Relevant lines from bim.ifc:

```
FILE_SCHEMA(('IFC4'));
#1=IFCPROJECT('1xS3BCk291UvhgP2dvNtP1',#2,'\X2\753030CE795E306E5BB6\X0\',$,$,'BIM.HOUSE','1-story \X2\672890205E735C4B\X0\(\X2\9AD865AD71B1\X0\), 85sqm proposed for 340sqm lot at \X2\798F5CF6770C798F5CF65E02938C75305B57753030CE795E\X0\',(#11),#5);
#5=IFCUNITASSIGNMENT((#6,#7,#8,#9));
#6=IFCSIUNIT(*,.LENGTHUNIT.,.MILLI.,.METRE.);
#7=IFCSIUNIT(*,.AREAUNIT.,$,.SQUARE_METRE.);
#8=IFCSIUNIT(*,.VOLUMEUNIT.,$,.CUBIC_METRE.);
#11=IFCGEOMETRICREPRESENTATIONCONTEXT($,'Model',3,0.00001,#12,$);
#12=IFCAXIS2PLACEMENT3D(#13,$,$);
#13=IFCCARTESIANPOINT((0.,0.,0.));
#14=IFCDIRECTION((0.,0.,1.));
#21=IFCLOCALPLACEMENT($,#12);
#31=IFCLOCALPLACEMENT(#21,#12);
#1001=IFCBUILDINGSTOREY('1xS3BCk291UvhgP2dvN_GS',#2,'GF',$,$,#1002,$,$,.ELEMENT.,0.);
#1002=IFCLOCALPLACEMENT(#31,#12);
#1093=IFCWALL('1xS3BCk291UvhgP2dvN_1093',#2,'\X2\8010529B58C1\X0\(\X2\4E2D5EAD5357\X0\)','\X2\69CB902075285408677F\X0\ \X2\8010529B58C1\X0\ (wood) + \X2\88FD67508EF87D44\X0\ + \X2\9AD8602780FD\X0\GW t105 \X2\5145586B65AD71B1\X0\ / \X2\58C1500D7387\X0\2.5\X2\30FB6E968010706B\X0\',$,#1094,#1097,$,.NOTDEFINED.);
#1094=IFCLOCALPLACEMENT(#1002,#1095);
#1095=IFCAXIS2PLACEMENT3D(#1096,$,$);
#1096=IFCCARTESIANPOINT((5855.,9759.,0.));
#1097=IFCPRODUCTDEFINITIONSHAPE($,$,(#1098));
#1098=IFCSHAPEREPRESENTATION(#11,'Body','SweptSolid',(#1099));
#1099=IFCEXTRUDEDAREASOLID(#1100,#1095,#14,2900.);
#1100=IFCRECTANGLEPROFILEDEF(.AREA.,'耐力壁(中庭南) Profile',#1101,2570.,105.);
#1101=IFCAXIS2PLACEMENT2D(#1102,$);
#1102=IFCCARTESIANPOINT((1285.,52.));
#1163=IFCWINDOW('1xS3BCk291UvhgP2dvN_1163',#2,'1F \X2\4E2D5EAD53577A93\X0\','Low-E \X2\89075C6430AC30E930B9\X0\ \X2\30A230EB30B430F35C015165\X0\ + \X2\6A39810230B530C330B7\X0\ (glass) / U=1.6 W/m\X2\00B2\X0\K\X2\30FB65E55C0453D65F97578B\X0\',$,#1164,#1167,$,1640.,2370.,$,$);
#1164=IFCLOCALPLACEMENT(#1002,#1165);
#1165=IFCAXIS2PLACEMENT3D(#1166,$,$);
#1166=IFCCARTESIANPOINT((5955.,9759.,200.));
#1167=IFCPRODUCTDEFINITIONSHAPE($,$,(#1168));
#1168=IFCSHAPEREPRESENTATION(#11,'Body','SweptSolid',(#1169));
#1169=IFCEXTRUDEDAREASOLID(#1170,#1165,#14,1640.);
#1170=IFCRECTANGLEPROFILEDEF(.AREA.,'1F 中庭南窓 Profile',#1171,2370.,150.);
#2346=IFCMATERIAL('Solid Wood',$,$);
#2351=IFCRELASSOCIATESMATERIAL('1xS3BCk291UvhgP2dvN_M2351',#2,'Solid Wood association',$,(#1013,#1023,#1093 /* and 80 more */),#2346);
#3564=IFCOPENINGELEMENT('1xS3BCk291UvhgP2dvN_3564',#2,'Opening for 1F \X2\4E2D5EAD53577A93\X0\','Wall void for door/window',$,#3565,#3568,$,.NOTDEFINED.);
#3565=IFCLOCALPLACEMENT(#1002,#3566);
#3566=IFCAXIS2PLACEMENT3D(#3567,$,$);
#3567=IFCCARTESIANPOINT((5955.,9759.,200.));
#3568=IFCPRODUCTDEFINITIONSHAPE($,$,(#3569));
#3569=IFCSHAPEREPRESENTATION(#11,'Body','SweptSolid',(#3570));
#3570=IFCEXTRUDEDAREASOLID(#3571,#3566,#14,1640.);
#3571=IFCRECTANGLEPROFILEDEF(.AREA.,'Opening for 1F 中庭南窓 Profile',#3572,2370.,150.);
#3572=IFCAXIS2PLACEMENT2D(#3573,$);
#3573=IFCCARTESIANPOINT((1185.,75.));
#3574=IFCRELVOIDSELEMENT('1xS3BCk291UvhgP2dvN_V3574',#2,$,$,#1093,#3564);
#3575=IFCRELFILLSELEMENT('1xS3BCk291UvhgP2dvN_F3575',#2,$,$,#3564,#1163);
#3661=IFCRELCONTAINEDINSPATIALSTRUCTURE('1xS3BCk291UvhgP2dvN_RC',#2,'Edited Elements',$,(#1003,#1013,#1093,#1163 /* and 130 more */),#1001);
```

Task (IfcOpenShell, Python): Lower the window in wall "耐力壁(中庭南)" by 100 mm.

```python
import numpy as np
import ifcopenshell
import ifcopenshell.api.geometry
import ifcopenshell.util.placement
import ifcopenshell.util.unit

model = ifcopenshell.open("bim.ifc")
unit_scale = ifcopenshell.util.unit.calculate_unit_scale(model)

window = model.by_guid("1xS3BCk291UvhgP2dvN_1163")
opening = window.FillsVoids[0].RelatingOpeningElement
dz = -0.1 / unit_scale

shift = np.array([0.0, 0.0, dz])
# The window is not placed relative to its opening, so move both.
for product in (opening, window):
    matrix = ifcopenshell.util.placement.get_local_placement(product.ObjectPlacement)
    matrix[:3, 3] += shift
    ifcopenshell.api.geometry.edit_object_placement(model, product=product, matrix=matrix, is_si=False)

print(f"moved by {dz * unit_scale:+.3f} m")

model.write("bim_v2.ifc")
```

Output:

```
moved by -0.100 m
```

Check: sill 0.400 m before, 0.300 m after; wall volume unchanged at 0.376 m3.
